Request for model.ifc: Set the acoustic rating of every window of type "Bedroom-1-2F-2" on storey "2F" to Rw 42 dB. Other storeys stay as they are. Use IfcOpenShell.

First a look at what the model holds.

```python
import ifcopenshell
import ifcopenshell.util.element

model = ifcopenshell.open("model.ifc")
print(model.schema)
storey = next(s for s in model.by_type("IfcBuildingStorey") if s.Name == "2F")
windows = [e for e in ifcopenshell.util.element.get_decomposition(storey) if e.is_a("IfcWindow")]
seen = {}
for e in windows:
    element_type = ifcopenshell.util.element.get_type(e)
    key = (element_type.Name if element_type != e and element_type else None, ifcopenshell.util.element.get_pset(e, "Pset_WindowCommon", "AcousticRating"))
    seen[key] = seen.get(key, 0) + 1
for (name, value), count in sorted(seen.items(), key=str):
    print(count, "x", name, "|", value)
```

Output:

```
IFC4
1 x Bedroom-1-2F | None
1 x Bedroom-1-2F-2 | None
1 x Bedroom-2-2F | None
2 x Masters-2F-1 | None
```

```python
import ifcopenshell
import ifcopenshell.api.pset
import ifcopenshell.util.element

model = ifcopenshell.open("model.ifc")

storey = next(s for s in model.by_type("IfcBuildingStorey") if s.Name == "2F")
windows = [e for e in ifcopenshell.util.element.get_decomposition(storey) if e.is_a("IfcWindow")]

count = 0
for e in windows:
    element_type = ifcopenshell.util.element.get_type(e)
    if element_type in (None, e) or element_type.Name != "Bedroom-1-2F-2":
        continue
    # add_pset returns the element's existing set when there is one.
    pset = ifcopenshell.api.pset.add_pset(model, product=e, name="Pset_WindowCommon")
    ifcopenshell.api.pset.edit_pset(model, pset=pset, properties={"AcousticRating": "Rw 42 dB"})
    count += 1

print(count, "windows updated")

model.write("model_v2.ifc")
```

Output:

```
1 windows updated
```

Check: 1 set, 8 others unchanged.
